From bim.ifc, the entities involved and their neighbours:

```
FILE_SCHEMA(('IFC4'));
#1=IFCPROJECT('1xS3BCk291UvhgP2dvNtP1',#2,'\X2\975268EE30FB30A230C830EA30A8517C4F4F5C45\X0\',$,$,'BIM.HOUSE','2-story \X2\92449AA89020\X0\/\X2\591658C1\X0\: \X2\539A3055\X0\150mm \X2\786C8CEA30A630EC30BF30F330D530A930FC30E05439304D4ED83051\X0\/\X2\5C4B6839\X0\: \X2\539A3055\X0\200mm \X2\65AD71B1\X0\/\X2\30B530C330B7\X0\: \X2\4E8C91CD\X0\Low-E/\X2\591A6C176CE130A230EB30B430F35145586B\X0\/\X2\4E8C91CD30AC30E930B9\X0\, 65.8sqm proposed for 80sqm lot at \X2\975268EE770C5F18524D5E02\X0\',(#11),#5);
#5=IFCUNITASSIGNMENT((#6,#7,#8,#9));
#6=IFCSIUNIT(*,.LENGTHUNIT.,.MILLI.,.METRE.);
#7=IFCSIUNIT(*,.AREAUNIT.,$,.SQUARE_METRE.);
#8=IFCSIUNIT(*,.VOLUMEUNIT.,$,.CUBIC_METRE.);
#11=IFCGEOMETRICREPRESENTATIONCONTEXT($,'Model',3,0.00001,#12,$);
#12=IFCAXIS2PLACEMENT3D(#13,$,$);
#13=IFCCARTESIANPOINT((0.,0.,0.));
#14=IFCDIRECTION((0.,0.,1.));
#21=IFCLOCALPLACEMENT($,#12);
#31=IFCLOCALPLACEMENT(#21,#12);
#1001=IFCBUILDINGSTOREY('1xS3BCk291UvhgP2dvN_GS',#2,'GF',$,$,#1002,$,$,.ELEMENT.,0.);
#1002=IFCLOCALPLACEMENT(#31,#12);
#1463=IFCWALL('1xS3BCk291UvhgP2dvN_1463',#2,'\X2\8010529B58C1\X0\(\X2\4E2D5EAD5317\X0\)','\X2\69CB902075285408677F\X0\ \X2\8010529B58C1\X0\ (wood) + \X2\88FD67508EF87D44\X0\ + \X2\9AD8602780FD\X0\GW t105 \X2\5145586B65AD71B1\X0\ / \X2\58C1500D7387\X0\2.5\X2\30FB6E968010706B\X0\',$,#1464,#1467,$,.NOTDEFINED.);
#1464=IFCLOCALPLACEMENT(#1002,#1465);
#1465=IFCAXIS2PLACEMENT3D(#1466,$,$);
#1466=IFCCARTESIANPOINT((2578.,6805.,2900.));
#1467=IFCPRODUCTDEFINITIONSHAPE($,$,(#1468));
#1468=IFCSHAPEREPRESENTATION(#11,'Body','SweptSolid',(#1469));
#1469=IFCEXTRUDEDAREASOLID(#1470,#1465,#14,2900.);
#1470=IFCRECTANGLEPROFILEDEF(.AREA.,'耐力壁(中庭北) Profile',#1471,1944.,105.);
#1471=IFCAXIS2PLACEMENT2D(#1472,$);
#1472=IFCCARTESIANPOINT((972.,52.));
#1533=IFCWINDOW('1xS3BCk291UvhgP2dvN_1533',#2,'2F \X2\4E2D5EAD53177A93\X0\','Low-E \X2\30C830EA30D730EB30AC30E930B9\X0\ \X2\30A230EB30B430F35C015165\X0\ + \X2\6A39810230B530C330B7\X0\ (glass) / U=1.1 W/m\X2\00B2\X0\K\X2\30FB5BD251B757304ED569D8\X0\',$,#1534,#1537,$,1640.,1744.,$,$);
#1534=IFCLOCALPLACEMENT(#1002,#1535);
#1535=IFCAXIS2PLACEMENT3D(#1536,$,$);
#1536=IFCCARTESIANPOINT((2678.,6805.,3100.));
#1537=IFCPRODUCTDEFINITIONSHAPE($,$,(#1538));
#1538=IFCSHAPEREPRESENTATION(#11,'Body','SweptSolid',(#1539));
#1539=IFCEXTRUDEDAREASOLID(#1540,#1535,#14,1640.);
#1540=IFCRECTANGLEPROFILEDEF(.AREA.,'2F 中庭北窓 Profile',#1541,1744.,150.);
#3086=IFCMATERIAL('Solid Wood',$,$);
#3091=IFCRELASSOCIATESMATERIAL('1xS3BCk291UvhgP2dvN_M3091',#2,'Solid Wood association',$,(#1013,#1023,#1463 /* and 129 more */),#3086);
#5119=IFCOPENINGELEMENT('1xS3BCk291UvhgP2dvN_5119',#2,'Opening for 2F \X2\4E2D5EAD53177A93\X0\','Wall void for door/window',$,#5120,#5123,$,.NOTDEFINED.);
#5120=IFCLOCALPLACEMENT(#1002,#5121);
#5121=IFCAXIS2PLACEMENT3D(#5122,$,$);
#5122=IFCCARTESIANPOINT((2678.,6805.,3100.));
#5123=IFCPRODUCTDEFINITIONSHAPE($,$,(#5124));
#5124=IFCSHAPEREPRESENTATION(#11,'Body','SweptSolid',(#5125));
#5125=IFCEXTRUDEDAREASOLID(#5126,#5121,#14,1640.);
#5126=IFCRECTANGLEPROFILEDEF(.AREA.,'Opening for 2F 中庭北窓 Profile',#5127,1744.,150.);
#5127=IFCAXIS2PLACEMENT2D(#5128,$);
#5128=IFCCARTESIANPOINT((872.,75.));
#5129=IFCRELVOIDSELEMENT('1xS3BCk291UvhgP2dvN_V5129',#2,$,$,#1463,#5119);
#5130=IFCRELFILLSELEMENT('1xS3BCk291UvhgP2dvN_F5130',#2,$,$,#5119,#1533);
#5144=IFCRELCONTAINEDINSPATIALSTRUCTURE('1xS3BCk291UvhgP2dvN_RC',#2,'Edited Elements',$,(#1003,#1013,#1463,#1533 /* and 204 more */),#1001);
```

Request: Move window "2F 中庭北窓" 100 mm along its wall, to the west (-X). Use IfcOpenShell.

```python
import ifcopenshell
import ifcopenshell.api.geometry
import ifcopenshell.util.placement

model = ifcopenshell.open("bim.ifc")

window = model.by_guid("1xS3BCk291UvhgP2dvN_1533")
opening = window.FillsVoids[0].RelatingOpeningElement
wall = opening.VoidsElements[0].RelatingBuildingElement

wall_matrix = ifcopenshell.util.placement.get_local_placement(wall.ObjectPlacement)
shift = wall_matrix[:3, 0] * -100.0
before = ifcopenshell.util.placement.get_local_placement(window.ObjectPlacement)[:3, 3].copy()

# The window is not placed relative to its opening, so move both.
for product in (opening, window):
    matrix = ifcopenshell.util.placement.get_local_placement(product.ObjectPlacement)
    matrix[:3, 3] += shift
    ifcopenshell.api.geometry.edit_object_placement(model, product=product, matrix=matrix, is_si=False)

after = ifcopenshell.util.placement.get_local_placement(window.ObjectPlacement)[:3, 3]
print("window moved by", (after - before).round(3) + 0.0)

model.write("bim-out.ifc")
```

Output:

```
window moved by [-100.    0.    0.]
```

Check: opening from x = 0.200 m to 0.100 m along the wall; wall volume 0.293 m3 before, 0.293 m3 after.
